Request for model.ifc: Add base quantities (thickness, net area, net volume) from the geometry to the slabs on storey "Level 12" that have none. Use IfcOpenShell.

First a look at what the model holds.

```python
import ifcopenshell
import ifcopenshell.util.element
import ifcopenshell.util.unit

model = ifcopenshell.open("model.ifc")
print(model.schema)
for unit_type in ("LENGTHUNIT", "AREAUNIT", "VOLUMEUNIT"):
    print(unit_type, ifcopenshell.util.unit.calculate_unit_scale(model, unit_type))
storey = next(s for s in model.by_type("IfcBuildingStorey") if s.Name == "Level 12")
slabs = [e for e in ifcopenshell.util.element.get_decomposition(storey) if e.is_a("IfcSlab")]
for e in sorted(slabs, key=lambda e: e.id()):
    print(e.id(), e.is_a(), e.Name, list(ifcopenshell.util.element.get_psets(e, qtos_only=True)), sep=" | ")
```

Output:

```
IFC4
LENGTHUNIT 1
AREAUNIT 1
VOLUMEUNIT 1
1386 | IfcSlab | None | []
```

```python
import ifcopenshell
import ifcopenshell.api.pset
import ifcopenshell.geom
import ifcopenshell.util.element
import ifcopenshell.util.shape
import ifcopenshell.util.unit

model = ifcopenshell.open("model.ifc")
unit_scale = ifcopenshell.util.unit.calculate_unit_scale(model)
area_scale = ifcopenshell.util.unit.calculate_unit_scale(model, "AREAUNIT")
volume_scale = ifcopenshell.util.unit.calculate_unit_scale(model, "VOLUMEUNIT")
settings = ifcopenshell.geom.settings()

storey = next(s for s in model.by_type("IfcBuildingStorey") if s.Name == "Level 12")
slabs = [e for e in ifcopenshell.util.element.get_decomposition(storey) if e.is_a("IfcSlab")]

for e in sorted(slabs, key=lambda e: e.id()):
    if ifcopenshell.util.element.get_psets(e, qtos_only=True, should_inherit=False):
        continue
    # Geometry comes back in metres, in the element's own axes.
    shape = ifcopenshell.geom.create_shape(settings, e)
    values = {
        "Width": ifcopenshell.util.shape.get_z(shape.geometry) / unit_scale,
        "NetArea": ifcopenshell.util.shape.get_footprint_area(shape.geometry) / area_scale,
        "NetVolume": ifcopenshell.util.shape.get_volume(shape.geometry) / volume_scale,
    }
    qto = ifcopenshell.api.pset.add_qto(model, product=e, name="Qto_SlabBaseQuantities")
    ifcopenshell.api.pset.edit_qto(model, qto=qto, properties=values)
    print(e.id(), {k: round(v, 3) for k, v in values.items()})

model.write("model_rev.ifc")
```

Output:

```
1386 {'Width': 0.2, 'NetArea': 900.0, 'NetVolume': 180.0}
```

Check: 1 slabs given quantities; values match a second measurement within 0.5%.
